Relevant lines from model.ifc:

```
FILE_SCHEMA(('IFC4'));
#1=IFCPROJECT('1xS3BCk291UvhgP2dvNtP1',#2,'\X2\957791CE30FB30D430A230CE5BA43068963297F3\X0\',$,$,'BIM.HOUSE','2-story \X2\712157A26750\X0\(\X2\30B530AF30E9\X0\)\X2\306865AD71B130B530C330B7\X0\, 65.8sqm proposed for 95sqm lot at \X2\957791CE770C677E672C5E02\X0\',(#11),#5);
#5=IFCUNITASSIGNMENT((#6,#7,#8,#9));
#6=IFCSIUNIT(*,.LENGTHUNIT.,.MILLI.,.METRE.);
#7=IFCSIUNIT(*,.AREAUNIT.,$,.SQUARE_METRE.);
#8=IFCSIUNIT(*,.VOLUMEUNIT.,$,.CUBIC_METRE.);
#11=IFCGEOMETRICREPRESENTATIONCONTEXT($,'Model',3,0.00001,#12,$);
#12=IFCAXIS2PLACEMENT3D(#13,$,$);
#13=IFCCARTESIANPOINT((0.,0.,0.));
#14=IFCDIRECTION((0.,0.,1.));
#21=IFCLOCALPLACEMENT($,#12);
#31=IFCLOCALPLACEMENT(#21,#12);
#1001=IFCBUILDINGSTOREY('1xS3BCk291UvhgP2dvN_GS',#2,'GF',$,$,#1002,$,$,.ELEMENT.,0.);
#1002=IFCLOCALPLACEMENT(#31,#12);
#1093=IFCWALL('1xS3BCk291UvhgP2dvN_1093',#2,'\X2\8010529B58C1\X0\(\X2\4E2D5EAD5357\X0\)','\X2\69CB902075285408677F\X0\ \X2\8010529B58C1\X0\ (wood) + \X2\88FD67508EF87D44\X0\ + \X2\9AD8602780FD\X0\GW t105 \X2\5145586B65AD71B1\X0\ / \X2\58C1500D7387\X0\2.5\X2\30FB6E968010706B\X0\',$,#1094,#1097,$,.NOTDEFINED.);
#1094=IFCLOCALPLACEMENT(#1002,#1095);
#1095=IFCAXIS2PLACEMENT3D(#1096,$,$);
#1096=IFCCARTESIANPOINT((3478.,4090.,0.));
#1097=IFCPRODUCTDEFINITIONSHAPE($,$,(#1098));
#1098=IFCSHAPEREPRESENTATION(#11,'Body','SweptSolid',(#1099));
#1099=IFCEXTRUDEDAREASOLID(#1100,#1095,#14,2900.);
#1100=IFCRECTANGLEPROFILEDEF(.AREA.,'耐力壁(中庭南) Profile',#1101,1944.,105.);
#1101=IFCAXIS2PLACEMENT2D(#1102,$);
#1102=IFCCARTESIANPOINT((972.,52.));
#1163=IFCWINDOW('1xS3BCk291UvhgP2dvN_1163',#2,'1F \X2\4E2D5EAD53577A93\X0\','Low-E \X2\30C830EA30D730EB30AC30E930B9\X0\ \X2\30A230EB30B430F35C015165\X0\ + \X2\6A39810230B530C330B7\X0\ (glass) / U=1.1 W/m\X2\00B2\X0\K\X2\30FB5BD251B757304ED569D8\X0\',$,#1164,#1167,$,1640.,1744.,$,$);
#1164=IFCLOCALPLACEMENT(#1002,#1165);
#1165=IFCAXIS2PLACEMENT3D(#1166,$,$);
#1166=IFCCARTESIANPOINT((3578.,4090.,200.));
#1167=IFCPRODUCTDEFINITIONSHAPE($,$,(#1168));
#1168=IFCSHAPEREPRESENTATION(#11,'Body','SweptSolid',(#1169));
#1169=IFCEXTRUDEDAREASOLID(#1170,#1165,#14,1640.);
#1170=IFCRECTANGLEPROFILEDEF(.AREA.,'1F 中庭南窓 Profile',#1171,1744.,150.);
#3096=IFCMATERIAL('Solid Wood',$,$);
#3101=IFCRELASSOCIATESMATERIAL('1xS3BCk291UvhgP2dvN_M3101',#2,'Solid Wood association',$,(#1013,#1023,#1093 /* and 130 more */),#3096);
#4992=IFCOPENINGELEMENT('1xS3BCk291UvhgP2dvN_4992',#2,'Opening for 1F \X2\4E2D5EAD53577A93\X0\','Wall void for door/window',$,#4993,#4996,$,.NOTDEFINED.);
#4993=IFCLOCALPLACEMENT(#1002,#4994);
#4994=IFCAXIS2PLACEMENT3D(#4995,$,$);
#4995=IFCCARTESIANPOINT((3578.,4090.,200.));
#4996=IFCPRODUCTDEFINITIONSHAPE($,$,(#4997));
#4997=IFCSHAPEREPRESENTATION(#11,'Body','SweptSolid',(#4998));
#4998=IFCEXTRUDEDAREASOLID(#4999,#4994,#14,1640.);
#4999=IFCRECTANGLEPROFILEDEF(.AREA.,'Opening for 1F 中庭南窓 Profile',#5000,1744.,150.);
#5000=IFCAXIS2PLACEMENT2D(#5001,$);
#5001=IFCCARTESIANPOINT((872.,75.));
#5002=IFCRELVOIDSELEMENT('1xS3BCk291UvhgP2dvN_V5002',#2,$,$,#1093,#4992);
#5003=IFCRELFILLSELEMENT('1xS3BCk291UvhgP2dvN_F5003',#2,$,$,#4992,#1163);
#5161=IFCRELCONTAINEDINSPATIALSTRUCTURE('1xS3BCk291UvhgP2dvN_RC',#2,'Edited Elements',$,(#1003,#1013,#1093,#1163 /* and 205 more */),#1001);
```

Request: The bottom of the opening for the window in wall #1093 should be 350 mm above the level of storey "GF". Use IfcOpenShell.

```python
import numpy as np
import ifcopenshell
import ifcopenshell.api.geometry
import ifcopenshell.geom
import ifcopenshell.util.element
import ifcopenshell.util.placement
import ifcopenshell.util.shape
import ifcopenshell.util.unit

model = ifcopenshell.open("model.ifc")
unit_scale = ifcopenshell.util.unit.calculate_unit_scale(model)

window = model.by_id(1163)
opening = window.FillsVoids[0].RelatingOpeningElement
storey = ifcopenshell.util.element.get_container(window, ifc_class="IfcBuildingStorey")
level = ifcopenshell.util.placement.get_local_placement(storey.ObjectPlacement)[2, 3]

# The opening's origin need not be at the sill, so measure its lowest point.
shape = ifcopenshell.geom.create_shape(ifcopenshell.geom.settings(), opening)
bottom = ifcopenshell.util.shape.get_shape_bottom_elevation(shape, shape.geometry) / unit_scale
dz = level + 0.35 / unit_scale - bottom

shift = np.array([0.0, 0.0, dz])
# The window is not placed relative to its opening, so move both.
for product in (opening, window):
    matrix = ifcopenshell.util.placement.get_local_placement(product.ObjectPlacement)
    matrix[:3, 3] += shift
    ifcopenshell.api.geometry.edit_object_placement(model, product=product, matrix=matrix, is_si=False)

print(f"moved by {dz * unit_scale:+.3f} m")

model.write("model_updated.ifc")
```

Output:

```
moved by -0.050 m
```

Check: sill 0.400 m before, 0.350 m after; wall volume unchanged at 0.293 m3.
